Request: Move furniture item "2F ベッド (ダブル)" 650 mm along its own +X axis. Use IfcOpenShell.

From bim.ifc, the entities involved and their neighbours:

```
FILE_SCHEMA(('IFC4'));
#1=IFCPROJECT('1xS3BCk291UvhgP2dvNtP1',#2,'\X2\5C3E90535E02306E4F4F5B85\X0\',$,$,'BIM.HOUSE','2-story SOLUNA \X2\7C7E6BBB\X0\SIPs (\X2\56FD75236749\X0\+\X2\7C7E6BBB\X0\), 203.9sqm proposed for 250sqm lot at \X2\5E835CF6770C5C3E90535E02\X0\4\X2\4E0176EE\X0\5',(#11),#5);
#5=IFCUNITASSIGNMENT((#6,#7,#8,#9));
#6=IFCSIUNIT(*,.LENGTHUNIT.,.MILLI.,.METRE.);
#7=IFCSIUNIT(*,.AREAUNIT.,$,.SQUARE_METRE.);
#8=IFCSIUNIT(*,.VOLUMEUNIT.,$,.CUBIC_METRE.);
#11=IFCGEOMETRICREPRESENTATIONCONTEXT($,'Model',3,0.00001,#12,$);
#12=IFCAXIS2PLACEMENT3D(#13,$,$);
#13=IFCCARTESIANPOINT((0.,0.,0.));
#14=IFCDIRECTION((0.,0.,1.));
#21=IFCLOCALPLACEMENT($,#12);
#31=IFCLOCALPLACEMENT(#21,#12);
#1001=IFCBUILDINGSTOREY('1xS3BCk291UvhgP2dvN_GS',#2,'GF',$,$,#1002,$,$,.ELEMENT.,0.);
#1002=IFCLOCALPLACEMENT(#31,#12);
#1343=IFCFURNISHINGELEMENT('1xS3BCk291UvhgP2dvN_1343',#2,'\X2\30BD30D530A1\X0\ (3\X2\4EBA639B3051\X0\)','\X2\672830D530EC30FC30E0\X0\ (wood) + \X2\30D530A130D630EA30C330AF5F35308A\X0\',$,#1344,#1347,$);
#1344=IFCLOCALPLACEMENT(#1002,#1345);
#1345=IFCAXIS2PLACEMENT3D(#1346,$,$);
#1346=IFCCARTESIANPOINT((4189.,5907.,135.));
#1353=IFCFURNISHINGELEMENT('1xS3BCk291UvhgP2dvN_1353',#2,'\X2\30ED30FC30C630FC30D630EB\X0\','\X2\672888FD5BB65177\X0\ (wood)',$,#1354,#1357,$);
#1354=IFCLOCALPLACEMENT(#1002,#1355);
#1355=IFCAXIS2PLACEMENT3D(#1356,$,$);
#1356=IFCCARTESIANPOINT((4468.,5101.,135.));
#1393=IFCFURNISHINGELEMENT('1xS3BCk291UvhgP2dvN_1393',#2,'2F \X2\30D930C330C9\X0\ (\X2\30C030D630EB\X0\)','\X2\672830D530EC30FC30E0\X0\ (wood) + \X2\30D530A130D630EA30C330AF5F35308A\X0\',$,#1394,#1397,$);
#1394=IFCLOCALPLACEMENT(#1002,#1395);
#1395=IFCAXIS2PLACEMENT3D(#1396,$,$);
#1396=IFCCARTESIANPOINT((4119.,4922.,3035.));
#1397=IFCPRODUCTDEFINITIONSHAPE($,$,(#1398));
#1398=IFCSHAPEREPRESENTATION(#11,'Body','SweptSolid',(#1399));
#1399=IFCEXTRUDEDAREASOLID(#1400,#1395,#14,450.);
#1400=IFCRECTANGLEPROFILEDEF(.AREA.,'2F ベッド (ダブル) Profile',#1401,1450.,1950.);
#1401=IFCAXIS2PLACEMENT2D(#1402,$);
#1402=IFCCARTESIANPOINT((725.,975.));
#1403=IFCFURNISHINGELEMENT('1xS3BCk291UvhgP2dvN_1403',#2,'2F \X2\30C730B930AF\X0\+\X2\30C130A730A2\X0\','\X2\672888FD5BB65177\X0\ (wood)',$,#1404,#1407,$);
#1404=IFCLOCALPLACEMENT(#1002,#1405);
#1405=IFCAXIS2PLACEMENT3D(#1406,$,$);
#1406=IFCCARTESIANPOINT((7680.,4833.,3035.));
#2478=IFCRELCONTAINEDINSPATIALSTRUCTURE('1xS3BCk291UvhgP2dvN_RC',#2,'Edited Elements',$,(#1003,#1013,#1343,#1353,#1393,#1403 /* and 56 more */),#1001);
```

```python
import ifcopenshell
import ifcopenshell.api.geometry
import ifcopenshell.util.placement
import ifcopenshell.util.unit

model = ifcopenshell.open("bim.ifc")
unit_scale = ifcopenshell.util.unit.calculate_unit_scale(model)

item = model.by_guid("1xS3BCk291UvhgP2dvN_1393")
matrix = ifcopenshell.util.placement.get_local_placement(item.ObjectPlacement)
matrix[:3, 3] += matrix[:3, 0] * 0.65 / unit_scale
ifcopenshell.api.geometry.edit_object_placement(model, product=item, matrix=matrix, is_si=False)

print(ifcopenshell.util.placement.get_local_placement(item.ObjectPlacement).round(3) + 0.0)

model.write("bim-out.ifc")
```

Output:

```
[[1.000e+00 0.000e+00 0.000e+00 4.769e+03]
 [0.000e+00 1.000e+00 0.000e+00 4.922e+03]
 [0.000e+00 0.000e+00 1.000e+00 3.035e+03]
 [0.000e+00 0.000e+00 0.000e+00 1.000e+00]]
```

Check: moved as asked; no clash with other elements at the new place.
